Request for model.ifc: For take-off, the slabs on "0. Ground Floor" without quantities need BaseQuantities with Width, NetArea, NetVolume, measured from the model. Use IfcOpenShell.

First a look at what the model holds.

```python
import ifcopenshell
import ifcopenshell.util.element
import ifcopenshell.util.unit

model = ifcopenshell.open("model.ifc")
print(model.schema)
for unit_type in ("LENGTHUNIT", "AREAUNIT", "VOLUMEUNIT"):
    print(unit_type, ifcopenshell.util.unit.calculate_unit_scale(model, unit_type))
storey = next(s for s in model.by_type("IfcBuildingStorey") if s.Name == "0. Ground Floor")
slabs = [e for e in ifcopenshell.util.element.get_decomposition(storey) if e.is_a("IfcSlab")]
for e in sorted(slabs, key=lambda e: e.id()):
    print(e.id(), e.is_a(), e.Name, list(ifcopenshell.util.element.get_psets(e, qtos_only=True)), sep=" | ")
```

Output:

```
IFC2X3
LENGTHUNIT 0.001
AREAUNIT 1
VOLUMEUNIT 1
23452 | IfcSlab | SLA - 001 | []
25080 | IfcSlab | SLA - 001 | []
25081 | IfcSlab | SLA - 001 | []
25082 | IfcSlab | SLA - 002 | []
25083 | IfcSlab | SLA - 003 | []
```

```python
import ifcopenshell
import ifcopenshell.api.pset
import ifcopenshell.geom
import ifcopenshell.util.element
import ifcopenshell.util.shape
import ifcopenshell.util.unit

model = ifcopenshell.open("model.ifc")
unit_scale = ifcopenshell.util.unit.calculate_unit_scale(model)
area_scale = ifcopenshell.util.unit.calculate_unit_scale(model, "AREAUNIT")
volume_scale = ifcopenshell.util.unit.calculate_unit_scale(model, "VOLUMEUNIT")
settings = ifcopenshell.geom.settings()

storey = next(s for s in model.by_type("IfcBuildingStorey") if s.Name == "0. Ground Floor")
slabs = [e for e in ifcopenshell.util.element.get_decomposition(storey) if e.is_a("IfcSlab")]

for e in sorted(slabs, key=lambda e: e.id()):
    if ifcopenshell.util.element.get_psets(e, qtos_only=True, should_inherit=False):
        continue
    # Geometry comes back in metres, in the element's own axes.
    shape = ifcopenshell.geom.create_shape(settings, e)
    values = {
        "Width": ifcopenshell.util.shape.get_z(shape.geometry) / unit_scale,
        "NetArea": ifcopenshell.util.shape.get_footprint_area(shape.geometry) / area_scale,
        "NetVolume": ifcopenshell.util.shape.get_volume(shape.geometry) / volume_scale,
    }
    qto = ifcopenshell.api.pset.add_qto(model, product=e, name="BaseQuantities")
    ifcopenshell.api.pset.edit_qto(model, qto=qto, properties=values)
    print(e.id(), {k: round(v, 3) for k, v in values.items()})

model.write("model_v2.ifc")
```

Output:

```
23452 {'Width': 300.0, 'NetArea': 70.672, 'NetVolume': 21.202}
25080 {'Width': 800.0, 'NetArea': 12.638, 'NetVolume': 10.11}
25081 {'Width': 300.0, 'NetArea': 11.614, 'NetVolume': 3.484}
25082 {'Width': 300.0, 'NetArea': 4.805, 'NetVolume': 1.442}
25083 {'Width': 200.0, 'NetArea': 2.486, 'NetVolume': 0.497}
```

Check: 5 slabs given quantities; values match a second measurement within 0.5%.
